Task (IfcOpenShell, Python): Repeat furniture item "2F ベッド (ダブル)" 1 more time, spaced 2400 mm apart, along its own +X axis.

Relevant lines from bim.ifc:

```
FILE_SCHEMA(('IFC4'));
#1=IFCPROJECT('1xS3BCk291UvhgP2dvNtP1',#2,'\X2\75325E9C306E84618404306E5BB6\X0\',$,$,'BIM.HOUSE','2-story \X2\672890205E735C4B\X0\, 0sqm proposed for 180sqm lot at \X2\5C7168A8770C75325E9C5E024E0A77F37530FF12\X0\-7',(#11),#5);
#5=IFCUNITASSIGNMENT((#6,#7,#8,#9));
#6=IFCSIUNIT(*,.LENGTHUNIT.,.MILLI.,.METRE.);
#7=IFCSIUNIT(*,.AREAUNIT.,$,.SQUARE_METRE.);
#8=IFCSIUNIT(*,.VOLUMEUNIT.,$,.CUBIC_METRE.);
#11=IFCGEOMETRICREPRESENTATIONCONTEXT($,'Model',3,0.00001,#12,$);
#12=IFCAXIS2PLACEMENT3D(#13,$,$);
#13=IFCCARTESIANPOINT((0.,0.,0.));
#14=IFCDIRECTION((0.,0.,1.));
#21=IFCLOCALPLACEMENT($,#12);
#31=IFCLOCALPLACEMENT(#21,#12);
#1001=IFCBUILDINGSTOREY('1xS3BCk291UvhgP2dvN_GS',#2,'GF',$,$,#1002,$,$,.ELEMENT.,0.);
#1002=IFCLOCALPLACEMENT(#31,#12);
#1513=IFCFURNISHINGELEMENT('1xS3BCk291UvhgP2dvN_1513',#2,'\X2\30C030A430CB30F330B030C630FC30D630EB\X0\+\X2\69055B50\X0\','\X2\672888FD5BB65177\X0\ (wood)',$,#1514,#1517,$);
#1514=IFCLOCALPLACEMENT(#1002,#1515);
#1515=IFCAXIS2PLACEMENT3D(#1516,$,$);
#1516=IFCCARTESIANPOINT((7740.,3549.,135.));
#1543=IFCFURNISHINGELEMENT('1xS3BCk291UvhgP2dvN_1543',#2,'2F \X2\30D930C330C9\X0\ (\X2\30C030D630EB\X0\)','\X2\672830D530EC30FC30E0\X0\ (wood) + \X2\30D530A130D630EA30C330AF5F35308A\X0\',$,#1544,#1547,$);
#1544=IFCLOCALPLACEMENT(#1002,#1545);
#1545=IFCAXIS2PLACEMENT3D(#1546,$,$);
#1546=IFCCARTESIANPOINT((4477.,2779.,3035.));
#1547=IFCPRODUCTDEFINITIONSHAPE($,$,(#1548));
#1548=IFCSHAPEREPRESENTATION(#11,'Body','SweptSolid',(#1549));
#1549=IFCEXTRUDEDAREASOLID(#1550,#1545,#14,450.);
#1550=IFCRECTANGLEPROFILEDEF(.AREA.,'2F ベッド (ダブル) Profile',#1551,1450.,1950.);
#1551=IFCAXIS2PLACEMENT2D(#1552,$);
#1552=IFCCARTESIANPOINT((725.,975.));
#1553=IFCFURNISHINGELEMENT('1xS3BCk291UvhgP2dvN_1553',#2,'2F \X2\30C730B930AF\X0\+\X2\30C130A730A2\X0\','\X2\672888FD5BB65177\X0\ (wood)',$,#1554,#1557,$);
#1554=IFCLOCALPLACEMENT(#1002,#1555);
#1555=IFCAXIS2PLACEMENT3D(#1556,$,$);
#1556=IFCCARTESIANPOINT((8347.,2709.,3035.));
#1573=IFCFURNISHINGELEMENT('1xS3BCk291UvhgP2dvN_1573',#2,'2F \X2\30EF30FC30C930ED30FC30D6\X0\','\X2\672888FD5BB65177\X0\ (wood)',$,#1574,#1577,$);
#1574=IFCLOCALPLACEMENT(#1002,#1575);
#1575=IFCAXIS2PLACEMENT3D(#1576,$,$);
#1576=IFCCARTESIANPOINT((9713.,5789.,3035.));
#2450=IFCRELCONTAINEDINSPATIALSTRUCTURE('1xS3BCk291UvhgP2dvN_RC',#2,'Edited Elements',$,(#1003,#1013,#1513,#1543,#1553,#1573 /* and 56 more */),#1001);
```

```python
import ifcopenshell
import ifcopenshell.api.geometry
import ifcopenshell.api.root
import ifcopenshell.util.element
import ifcopenshell.util.placement
import ifcopenshell.util.unit

model = ifcopenshell.open("bim.ifc")
unit_scale = ifcopenshell.util.unit.calculate_unit_scale(model)


def reuse_history(source, copy):
    """copy_class also copies each property set's owner history, people and application; keep the originals."""
    for rel in copy.IsDefinedBy:
        if rel.is_a("IfcRelDefinesByProperties") and (history := rel.RelatingPropertyDefinition.OwnerHistory):
            rel.RelatingPropertyDefinition.OwnerHistory = source.OwnerHistory
            ifcopenshell.util.element.remove_deep2(model, history)


source = model.by_guid("1xS3BCk291UvhgP2dvN_1543")
base = ifcopenshell.util.placement.get_local_placement(source.ObjectPlacement)
step = base[:3, 0] * 2.4 / unit_scale

for i in range(1, 2):
    copy = ifcopenshell.api.root.copy_class(model, product=source)
    copy.Representation = ifcopenshell.util.element.copy_deep(
        model, source.Representation, exclude=["IfcGeometricRepresentationContext", "IfcRepresentationMap"]
    )
    reuse_history(source, copy)
    matrix = base.copy()
    matrix[:3, 3] += i * step
    print("added at", matrix[:3, 3].round(3) + 0.0)
    ifcopenshell.api.geometry.edit_object_placement(model, product=copy, matrix=matrix, is_si=False)

model.write("bim_edited.ifc")
```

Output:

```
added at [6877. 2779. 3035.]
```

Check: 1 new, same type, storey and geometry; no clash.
